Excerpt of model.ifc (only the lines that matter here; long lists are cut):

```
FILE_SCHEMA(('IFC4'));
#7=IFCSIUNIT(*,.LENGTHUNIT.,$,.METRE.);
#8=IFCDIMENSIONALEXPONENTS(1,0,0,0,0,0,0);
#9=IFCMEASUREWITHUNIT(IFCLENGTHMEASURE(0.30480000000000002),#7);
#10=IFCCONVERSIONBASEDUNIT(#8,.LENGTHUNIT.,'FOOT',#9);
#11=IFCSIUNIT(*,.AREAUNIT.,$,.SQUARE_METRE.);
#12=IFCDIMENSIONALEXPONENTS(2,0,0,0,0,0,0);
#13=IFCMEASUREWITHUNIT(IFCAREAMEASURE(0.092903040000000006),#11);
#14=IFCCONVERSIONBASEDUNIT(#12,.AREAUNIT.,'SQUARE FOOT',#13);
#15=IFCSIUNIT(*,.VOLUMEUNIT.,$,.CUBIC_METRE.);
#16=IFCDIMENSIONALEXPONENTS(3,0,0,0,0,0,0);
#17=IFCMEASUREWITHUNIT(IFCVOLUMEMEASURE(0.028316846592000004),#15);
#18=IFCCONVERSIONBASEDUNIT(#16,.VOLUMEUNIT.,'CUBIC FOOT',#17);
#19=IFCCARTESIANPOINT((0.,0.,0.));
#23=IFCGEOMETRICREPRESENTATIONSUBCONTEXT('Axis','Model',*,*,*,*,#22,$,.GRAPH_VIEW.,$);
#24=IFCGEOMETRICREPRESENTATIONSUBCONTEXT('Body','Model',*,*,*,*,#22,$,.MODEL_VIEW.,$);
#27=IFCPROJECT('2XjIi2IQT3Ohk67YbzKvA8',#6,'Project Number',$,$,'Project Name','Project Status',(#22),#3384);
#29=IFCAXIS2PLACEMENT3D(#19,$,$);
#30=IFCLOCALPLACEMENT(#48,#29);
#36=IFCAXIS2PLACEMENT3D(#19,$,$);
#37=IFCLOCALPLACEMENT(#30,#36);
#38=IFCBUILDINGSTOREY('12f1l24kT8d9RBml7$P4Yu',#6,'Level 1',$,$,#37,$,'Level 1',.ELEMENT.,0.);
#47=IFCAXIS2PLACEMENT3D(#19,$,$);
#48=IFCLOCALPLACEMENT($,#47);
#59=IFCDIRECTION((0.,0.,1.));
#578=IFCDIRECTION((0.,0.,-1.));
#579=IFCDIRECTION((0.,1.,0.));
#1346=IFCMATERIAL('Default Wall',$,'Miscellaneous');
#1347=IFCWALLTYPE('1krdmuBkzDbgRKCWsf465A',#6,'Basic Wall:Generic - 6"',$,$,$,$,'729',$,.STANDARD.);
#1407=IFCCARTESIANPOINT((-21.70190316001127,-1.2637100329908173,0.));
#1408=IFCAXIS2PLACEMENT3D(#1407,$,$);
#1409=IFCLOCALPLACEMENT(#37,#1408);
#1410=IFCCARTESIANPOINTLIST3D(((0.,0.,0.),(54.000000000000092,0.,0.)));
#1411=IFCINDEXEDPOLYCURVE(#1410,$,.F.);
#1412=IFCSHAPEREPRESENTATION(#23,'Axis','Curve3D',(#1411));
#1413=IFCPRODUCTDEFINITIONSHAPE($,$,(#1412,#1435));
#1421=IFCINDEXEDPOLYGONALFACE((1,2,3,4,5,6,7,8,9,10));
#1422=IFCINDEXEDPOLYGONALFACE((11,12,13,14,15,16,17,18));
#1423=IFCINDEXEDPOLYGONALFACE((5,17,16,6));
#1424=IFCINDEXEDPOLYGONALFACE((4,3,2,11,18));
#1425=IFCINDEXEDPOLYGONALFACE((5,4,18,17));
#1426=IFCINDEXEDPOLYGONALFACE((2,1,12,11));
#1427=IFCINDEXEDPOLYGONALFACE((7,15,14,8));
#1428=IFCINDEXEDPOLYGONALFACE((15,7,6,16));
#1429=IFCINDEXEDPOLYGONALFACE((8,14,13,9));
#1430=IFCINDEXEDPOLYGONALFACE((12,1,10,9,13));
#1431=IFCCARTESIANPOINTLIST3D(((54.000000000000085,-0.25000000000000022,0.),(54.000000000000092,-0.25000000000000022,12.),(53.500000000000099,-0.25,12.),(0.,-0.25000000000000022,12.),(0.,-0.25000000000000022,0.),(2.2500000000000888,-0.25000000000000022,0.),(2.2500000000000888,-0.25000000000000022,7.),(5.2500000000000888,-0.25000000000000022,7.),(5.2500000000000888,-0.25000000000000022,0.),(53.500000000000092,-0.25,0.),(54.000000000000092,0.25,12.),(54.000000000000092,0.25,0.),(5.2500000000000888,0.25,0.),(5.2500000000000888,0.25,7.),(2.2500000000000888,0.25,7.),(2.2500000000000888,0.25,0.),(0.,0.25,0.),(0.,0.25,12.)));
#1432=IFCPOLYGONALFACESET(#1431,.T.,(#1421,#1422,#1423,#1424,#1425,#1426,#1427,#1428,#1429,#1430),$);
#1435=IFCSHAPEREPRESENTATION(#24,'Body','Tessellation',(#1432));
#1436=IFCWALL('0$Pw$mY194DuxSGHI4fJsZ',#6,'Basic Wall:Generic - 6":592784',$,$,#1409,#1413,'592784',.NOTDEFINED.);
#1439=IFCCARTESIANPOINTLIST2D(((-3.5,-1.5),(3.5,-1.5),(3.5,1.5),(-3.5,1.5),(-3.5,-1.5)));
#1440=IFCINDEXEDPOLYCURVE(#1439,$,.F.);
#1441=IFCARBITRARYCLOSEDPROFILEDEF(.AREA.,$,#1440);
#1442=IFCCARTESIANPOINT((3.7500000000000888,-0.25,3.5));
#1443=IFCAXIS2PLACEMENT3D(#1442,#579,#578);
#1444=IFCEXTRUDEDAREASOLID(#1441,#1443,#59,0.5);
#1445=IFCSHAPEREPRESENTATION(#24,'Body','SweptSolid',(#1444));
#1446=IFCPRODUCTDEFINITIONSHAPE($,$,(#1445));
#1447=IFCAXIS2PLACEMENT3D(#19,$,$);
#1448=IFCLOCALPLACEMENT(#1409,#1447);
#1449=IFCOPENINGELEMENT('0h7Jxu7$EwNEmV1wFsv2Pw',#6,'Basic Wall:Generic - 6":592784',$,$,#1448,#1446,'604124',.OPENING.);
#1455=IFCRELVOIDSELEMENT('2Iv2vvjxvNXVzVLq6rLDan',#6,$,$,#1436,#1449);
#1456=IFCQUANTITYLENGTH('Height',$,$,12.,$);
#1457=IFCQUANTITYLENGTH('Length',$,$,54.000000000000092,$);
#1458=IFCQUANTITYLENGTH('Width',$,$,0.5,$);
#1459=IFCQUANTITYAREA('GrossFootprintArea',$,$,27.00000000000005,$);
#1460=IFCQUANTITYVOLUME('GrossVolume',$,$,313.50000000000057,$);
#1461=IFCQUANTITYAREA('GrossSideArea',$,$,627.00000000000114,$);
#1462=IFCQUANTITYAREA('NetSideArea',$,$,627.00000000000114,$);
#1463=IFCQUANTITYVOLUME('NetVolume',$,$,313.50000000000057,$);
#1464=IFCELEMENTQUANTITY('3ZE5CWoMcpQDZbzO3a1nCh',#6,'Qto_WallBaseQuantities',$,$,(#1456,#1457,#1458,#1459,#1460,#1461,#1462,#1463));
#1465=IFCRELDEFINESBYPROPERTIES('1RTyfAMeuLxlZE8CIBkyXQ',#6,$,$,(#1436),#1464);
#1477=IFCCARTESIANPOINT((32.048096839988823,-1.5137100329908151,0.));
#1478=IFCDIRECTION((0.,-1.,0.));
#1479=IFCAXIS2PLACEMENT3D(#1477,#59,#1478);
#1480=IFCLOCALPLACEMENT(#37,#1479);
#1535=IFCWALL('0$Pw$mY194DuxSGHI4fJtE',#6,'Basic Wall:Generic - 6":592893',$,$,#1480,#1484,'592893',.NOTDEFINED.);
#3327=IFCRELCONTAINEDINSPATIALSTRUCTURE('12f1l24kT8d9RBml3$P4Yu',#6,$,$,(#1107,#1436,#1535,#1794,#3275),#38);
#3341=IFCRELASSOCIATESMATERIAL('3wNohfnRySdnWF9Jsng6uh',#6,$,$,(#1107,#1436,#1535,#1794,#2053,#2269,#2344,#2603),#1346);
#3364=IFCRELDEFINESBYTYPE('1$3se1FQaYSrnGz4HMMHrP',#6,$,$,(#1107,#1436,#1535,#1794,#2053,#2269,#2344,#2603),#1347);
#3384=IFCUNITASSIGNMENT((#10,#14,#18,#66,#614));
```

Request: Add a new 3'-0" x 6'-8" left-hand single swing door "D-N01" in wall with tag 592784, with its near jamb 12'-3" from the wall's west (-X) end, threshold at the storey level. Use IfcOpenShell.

```python
import numpy as np
import ifcopenshell
import ifcopenshell.api.feature
import ifcopenshell.api.geometry
import ifcopenshell.api.pset
import ifcopenshell.api.root
import ifcopenshell.api.spatial
import ifcopenshell.geom
import ifcopenshell.util.element
import ifcopenshell.util.placement
import ifcopenshell.util.representation
import ifcopenshell.util.shape
import ifcopenshell.util.unit

model = ifcopenshell.open("model.ifc")
unit_scale = ifcopenshell.util.unit.calculate_unit_scale(model)
area_scale = ifcopenshell.util.unit.calculate_unit_scale(model, "AREAUNIT")
volume_scale = ifcopenshell.util.unit.calculate_unit_scale(model, "VOLUMEUNIT")
settings = ifcopenshell.geom.settings()


def volume(element):
    """Net volume in cubic metres, openings subtracted."""
    shape = ifcopenshell.geom.create_shape(settings, element)
    return ifcopenshell.util.shape.get_volume(shape.geometry)


wall = model.by_guid("0$Pw$mY194DuxSGHI4fJsZ")
storey = ifcopenshell.util.element.get_container(wall, ifc_class="IfcBuildingStorey")
context = ifcopenshell.util.representation.get_context(model, "Model", "Body", "MODEL_VIEW")
before = volume(wall)

width, height, from_end, sill = 0.9144, 2.032, 3.7338, 0.0  # metres

# The wall runs along its own X axis, and the end named is its -X end.
wall_shape = ifcopenshell.geom.create_shape(settings, wall)
x, y, z = ifcopenshell.util.shape.get_vertices(wall_shape.geometry).T
start = x.min() + from_end
face, thickness = float(y.min()), float(y.max() - y.min())
wall_matrix = ifcopenshell.util.placement.get_local_placement(wall.ObjectPlacement)
level = ifcopenshell.util.placement.get_local_placement(storey.ObjectPlacement)[2, 3]


def in_wall(x, y):
    """Placement at x, y metres in the wall's axes, at sill height."""
    matrix = wall_matrix.copy()
    matrix[:, 3] = wall_matrix @ np.array([x / unit_scale, y / unit_scale, 0.0, 1.0])
    matrix[2, 3] = level + sill / unit_scale
    return matrix


# Opening: a box that overshoots both wall faces by 50 mm.
opening = ifcopenshell.api.root.create_entity(model, ifc_class="IfcOpeningElement", predefined_type="OPENING")
box = ifcopenshell.api.geometry.add_wall_representation(
    model, context=context, length=width, height=height, thickness=thickness + 0.1
)
ifcopenshell.api.geometry.assign_representation(model, product=opening, representation=box)
ifcopenshell.api.geometry.edit_object_placement(model, product=opening, matrix=in_wall(start, face - 0.05), is_si=False)
ifcopenshell.api.feature.add_feature(model, feature=opening, element=wall)

door = ifcopenshell.api.root.create_entity(model, ifc_class="IfcDoor", name="D-N01", predefined_type="DOOR")
door.OverallWidth, door.OverallHeight = width / unit_scale, height / unit_scale
door.OperationType = "SINGLE_SWING_LEFT"
body = ifcopenshell.api.geometry.add_door_representation(
    model,
    context=context,
    overall_width=door.OverallWidth,
    overall_height=door.OverallHeight,
    operation_type="SINGLE_SWING_LEFT",
    lining_properties={"LiningDepth": thickness / unit_scale, "ThresholdDepth": thickness / unit_scale},
)
ifcopenshell.api.geometry.assign_representation(model, product=door, representation=body)
ifcopenshell.api.spatial.assign_container(model, products=[door], relating_structure=storey)
ifcopenshell.api.feature.add_filling(model, opening=opening, element=door)

# The lining spans the wall, so the door starts at the wall face.
ifcopenshell.api.geometry.edit_object_placement(model, product=door, matrix=in_wall(start, face), is_si=False)

after = volume(wall)

# Update the wall's stored quantities.
qto = model.by_id(ifcopenshell.util.element.get_pset(wall, "Qto_WallBaseQuantities", should_inherit=False)["id"])
ifcopenshell.api.pset.edit_qto(model, qto=qto, properties={
    "NetSideArea": after / thickness / area_scale,
    "NetVolume": after / volume_scale,
})

print(f"wall volume {before:.3f} -> {after:.3f} m3")

model.write("model_edited.ifc")
```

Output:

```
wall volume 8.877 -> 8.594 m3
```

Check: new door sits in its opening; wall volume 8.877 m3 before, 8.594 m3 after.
